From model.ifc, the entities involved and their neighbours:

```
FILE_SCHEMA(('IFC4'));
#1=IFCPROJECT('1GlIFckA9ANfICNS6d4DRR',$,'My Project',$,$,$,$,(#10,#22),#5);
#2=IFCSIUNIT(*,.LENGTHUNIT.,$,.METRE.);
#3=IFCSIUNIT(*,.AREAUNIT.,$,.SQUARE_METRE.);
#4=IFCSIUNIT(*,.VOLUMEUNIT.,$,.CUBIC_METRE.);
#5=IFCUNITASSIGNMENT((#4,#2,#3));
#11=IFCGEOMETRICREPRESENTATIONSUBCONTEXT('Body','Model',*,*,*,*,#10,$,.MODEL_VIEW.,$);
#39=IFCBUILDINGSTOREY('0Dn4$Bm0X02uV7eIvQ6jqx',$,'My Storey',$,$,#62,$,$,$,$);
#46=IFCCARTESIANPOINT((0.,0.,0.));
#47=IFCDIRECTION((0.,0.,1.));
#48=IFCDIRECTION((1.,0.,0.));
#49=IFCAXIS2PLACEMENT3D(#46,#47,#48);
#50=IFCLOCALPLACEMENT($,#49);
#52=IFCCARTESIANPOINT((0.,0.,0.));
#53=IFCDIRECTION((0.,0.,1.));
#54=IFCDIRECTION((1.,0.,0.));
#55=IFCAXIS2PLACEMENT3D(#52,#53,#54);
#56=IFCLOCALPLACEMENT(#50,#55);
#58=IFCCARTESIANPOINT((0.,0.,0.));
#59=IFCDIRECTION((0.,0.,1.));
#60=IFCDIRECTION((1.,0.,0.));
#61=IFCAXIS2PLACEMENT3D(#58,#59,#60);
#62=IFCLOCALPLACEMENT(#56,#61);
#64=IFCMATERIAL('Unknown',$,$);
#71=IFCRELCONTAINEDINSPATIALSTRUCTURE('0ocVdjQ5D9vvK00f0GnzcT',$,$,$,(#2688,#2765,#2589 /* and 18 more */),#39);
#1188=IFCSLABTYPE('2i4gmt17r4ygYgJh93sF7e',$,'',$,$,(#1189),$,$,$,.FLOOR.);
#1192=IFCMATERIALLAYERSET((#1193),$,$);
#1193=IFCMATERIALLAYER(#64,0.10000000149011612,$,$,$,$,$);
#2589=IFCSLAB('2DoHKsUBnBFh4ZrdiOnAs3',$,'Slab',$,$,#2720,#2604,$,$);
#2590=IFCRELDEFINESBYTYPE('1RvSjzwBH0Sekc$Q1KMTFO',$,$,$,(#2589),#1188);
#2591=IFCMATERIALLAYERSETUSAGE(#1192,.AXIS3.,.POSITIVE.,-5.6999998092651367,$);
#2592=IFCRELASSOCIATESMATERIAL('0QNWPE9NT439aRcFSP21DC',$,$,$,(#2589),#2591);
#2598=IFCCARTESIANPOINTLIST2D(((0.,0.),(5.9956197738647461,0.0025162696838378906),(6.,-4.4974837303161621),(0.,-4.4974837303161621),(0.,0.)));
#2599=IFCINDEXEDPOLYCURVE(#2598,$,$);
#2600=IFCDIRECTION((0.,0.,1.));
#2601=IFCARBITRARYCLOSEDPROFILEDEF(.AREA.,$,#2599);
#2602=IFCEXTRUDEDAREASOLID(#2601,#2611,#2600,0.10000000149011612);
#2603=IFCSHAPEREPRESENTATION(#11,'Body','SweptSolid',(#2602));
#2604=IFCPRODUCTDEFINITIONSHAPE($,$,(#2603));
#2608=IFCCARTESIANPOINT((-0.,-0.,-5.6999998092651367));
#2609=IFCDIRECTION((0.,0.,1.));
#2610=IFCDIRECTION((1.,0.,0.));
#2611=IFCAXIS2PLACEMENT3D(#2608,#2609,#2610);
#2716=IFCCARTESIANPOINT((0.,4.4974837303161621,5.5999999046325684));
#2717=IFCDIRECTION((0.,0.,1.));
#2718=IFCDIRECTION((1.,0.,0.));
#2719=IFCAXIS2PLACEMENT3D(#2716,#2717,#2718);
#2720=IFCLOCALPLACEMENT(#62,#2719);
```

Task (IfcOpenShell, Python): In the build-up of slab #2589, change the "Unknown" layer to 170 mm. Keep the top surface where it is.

```python
import ifcopenshell
import ifcopenshell.util.element
import ifcopenshell.util.representation

model = ifcopenshell.open("model.ifc")

layer_set = model.by_id(1192)
layer = next(l for l in layer_set.MaterialLayers if l.Material and l.Material.Name == "Unknown")
change = 0.17 - layer.LayerThickness
layer.LayerThickness += change

# Geometry does not follow the layer set by itself.
slabs = [e for e in ifcopenshell.util.element.get_elements_by_material(model, layer_set) if e.is_a("IfcSlab")]
for slab in sorted(slabs, key=lambda e: e.id()):
    body = ifcopenshell.util.representation.get_representation(slab, "Model", "Body")
    solid = body.Items[0]
    old_depth = solid.Depth
    solid.Depth += change
    # Extruded upwards: lower the start of the extrusion so the top stays.
    x, y, z = solid.Position.Location.Coordinates
    solid.Position.Location = model.createIfcCartesianPoint((x, y, z - change))
    print(slab.id(), f"{old_depth:g} -> {solid.Depth:g}")

# The layers are counted up from the underside, which has moved.
for usage in {ifcopenshell.util.element.get_material(slab) for slab in slabs}:
    usage.OffsetFromReferenceLine -= change

model.write("model_rev.ifc")
```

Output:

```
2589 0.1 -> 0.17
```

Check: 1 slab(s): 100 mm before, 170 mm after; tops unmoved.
